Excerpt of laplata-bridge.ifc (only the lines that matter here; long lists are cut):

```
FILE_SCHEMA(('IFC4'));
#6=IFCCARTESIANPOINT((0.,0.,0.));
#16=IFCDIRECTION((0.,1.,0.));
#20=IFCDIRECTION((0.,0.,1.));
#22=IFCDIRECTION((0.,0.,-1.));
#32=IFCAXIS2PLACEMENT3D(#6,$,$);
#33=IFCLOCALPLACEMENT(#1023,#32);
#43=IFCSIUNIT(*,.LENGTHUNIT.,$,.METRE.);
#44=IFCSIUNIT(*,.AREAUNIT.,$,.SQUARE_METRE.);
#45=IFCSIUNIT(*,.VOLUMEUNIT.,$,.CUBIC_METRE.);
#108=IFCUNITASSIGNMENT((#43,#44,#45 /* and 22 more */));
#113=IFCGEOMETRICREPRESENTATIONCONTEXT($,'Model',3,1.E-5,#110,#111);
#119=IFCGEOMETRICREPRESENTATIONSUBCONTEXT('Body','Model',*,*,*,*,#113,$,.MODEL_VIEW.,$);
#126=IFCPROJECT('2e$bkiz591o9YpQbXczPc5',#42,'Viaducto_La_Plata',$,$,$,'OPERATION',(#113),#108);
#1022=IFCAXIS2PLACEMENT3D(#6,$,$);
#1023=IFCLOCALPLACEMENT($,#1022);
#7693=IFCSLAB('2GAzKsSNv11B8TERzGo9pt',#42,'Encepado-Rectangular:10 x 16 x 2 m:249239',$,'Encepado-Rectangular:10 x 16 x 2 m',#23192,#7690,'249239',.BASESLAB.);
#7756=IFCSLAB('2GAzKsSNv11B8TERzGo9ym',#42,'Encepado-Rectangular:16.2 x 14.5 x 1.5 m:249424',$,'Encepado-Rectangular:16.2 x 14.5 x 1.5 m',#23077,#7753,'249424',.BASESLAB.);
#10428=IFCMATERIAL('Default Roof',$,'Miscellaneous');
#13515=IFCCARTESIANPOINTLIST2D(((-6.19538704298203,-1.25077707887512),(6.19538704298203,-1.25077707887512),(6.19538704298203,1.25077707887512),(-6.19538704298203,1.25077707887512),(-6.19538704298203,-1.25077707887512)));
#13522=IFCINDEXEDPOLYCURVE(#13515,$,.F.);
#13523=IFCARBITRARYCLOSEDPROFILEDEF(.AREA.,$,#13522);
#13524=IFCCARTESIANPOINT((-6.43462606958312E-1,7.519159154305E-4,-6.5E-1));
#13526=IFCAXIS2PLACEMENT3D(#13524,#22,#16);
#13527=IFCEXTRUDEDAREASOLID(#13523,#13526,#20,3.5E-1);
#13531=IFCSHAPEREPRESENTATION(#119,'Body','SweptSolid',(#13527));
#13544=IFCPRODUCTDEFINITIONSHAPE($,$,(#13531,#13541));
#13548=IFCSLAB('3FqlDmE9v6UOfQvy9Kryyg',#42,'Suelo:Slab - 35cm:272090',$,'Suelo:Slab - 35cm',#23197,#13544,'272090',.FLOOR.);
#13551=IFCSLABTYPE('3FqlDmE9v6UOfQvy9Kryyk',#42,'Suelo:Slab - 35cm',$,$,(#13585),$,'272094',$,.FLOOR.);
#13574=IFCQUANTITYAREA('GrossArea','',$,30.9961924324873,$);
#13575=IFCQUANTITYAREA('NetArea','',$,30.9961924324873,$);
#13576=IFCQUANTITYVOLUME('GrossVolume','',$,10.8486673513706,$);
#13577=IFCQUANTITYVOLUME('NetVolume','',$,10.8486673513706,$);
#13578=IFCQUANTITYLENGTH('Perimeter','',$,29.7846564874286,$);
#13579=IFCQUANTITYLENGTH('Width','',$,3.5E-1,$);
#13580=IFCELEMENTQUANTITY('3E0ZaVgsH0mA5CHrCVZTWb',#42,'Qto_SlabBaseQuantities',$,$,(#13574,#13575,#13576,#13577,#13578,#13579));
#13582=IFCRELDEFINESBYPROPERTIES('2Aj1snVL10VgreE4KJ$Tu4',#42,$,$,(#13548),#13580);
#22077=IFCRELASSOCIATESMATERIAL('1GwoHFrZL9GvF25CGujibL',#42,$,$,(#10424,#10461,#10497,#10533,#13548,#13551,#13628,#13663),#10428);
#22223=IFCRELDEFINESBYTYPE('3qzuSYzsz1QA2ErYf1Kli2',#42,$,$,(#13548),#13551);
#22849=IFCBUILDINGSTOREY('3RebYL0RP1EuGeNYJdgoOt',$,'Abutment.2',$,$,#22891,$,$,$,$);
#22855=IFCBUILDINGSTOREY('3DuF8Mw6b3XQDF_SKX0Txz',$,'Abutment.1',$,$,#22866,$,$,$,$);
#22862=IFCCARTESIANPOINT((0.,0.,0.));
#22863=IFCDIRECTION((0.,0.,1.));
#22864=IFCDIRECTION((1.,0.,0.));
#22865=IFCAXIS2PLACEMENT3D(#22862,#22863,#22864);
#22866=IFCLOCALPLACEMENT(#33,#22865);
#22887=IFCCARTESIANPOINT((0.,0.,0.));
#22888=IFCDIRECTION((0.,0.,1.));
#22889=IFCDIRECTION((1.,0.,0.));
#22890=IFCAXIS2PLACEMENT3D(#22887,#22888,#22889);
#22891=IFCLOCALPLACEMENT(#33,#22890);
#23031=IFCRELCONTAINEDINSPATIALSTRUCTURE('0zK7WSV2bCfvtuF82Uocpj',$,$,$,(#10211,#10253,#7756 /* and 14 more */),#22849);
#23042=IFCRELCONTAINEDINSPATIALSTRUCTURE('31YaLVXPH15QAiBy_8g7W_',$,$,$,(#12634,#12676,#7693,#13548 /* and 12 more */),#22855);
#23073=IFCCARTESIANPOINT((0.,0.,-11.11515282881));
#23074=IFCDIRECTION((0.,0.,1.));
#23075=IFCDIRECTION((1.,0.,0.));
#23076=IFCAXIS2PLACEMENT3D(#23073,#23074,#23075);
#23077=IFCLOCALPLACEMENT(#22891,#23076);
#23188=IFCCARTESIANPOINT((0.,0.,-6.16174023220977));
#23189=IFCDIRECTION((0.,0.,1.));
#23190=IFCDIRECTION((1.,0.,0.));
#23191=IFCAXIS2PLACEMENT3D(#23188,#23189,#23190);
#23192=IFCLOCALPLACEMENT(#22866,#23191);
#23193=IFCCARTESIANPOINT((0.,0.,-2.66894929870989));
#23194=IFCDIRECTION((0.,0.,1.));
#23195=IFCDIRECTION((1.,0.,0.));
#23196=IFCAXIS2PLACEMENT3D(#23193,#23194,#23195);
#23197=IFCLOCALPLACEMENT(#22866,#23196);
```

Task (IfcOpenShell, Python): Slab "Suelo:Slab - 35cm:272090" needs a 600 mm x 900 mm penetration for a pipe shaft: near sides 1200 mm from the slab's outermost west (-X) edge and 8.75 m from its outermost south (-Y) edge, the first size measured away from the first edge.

```python
import numpy as np
import ifcopenshell
import ifcopenshell.api.feature
import ifcopenshell.api.geometry
import ifcopenshell.api.pset
import ifcopenshell.api.root
import ifcopenshell.geom
import ifcopenshell.util.element
import ifcopenshell.util.placement
import ifcopenshell.util.representation
import ifcopenshell.util.shape
import ifcopenshell.util.unit

model = ifcopenshell.open("laplata-bridge.ifc")
unit_scale = ifcopenshell.util.unit.calculate_unit_scale(model)
area_scale = ifcopenshell.util.unit.calculate_unit_scale(model, "AREAUNIT")
volume_scale = ifcopenshell.util.unit.calculate_unit_scale(model, "VOLUMEUNIT")
settings = ifcopenshell.geom.settings()


def volume(element):
    """Net volume in cubic metres, openings subtracted."""
    shape = ifcopenshell.geom.create_shape(settings, element)
    return ifcopenshell.util.shape.get_volume(shape.geometry)


slab = model.by_id(13548)
before = volume(slab)

# Extent in the slab's own axes, in metres. The edges named are its -X and -Y sides.
slab_shape = ifcopenshell.geom.create_shape(settings, slab)
vertices = ifcopenshell.util.shape.get_vertices(slab_shape.geometry)
x_min, y_min, bottom = vertices.min(axis=0)
top = vertices[:, 2].max()

opening = ifcopenshell.api.root.create_entity(model, ifc_class="IfcOpeningElement", name="Pipe shaft opening", predefined_type="OPENING")
context = ifcopenshell.util.representation.get_context(model, "Model", "Body", "MODEL_VIEW")
width, depth = 0.6, 0.9
outline = [(0.0, 0.0), (width, 0.0), (width, depth), (0.0, depth), (0.0, 0.0)]
# Overshoot both faces by 50 mm so the cut is clean.
shape = ifcopenshell.api.geometry.add_slab_representation(
    model, context=context, depth=top - bottom + 0.1, polyline=outline
)
ifcopenshell.api.geometry.assign_representation(model, product=opening, representation=shape)

matrix = ifcopenshell.util.placement.get_local_placement(slab.ObjectPlacement)
matrix[:, 3] = matrix @ np.append(np.array([x_min + 1.2, y_min + 8.75, bottom - 0.05]) / unit_scale, 1.0)
ifcopenshell.api.geometry.edit_object_placement(model, product=opening, matrix=matrix, is_si=False)
ifcopenshell.api.feature.add_feature(model, feature=opening, element=slab)

after = volume(slab)

# Update the slab's stored quantities.
qto = model.by_id(ifcopenshell.util.element.get_pset(slab, "Qto_SlabBaseQuantities", should_inherit=False)["id"])
ifcopenshell.api.pset.edit_qto(model, qto=qto, properties={
    "NetArea": after / (top - bottom) / area_scale,
    "NetVolume": after / volume_scale,
})

print(f"slab volume {before:.3f} -> {after:.3f} m3")

model.write("laplata-bridge_updated.ifc")
```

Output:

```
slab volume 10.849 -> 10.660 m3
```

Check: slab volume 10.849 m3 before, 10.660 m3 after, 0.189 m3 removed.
